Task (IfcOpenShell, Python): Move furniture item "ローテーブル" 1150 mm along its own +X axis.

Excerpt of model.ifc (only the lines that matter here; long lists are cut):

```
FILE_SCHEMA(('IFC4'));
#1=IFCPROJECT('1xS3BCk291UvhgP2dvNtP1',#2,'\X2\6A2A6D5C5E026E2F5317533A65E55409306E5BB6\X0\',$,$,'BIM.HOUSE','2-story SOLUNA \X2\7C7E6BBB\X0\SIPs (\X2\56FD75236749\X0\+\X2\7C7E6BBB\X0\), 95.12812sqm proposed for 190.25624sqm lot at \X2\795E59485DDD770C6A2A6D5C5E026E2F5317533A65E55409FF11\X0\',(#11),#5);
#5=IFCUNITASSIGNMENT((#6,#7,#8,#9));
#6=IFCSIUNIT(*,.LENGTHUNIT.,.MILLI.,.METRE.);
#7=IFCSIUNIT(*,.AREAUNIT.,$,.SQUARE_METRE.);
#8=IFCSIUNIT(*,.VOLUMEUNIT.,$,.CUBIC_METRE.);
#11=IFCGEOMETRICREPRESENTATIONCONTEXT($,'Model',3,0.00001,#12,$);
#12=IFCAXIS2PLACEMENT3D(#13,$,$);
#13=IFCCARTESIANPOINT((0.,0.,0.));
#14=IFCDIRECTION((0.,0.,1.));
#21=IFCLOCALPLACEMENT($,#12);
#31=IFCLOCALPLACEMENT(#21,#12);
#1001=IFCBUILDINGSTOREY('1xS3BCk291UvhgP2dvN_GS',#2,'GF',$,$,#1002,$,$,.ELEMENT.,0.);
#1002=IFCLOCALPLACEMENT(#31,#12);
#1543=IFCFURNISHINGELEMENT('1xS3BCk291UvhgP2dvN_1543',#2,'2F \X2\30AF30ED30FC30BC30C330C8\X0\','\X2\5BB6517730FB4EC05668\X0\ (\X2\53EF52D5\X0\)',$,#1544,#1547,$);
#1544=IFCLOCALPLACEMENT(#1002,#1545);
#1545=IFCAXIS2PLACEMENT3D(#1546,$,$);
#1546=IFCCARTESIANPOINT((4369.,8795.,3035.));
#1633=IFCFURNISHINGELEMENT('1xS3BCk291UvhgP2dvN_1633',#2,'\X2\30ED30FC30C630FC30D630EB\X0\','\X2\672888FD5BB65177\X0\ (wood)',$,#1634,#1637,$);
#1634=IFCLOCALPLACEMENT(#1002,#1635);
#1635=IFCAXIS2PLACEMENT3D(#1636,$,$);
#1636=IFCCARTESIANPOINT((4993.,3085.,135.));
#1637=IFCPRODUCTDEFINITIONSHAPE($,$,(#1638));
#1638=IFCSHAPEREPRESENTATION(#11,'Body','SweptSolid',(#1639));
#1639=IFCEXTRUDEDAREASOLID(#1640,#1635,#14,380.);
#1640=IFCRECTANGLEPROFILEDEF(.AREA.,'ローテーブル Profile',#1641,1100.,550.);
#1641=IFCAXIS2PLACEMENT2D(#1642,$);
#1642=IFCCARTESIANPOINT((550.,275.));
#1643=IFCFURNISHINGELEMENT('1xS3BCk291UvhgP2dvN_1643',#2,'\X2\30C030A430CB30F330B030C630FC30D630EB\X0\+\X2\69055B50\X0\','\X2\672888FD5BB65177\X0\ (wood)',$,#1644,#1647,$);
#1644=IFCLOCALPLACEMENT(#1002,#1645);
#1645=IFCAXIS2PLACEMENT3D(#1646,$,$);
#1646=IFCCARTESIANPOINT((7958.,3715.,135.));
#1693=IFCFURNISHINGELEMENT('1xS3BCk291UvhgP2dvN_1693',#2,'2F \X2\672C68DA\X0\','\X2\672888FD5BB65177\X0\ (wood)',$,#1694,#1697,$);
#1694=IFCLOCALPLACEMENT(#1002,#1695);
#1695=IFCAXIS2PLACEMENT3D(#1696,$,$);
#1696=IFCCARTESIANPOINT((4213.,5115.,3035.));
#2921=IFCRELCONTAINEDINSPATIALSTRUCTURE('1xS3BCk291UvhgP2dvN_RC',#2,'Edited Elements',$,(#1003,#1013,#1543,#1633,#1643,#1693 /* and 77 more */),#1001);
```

```python
import ifcopenshell
import ifcopenshell.api.geometry
import ifcopenshell.util.placement
import ifcopenshell.util.unit

model = ifcopenshell.open("model.ifc")
unit_scale = ifcopenshell.util.unit.calculate_unit_scale(model)

item = model.by_id(1633)
matrix = ifcopenshell.util.placement.get_local_placement(item.ObjectPlacement)
matrix[:3, 3] += matrix[:3, 0] * 1.15 / unit_scale
ifcopenshell.api.geometry.edit_object_placement(model, product=item, matrix=matrix, is_si=False)

print(ifcopenshell.util.placement.get_local_placement(item.ObjectPlacement).round(3) + 0.0)

model.write("model_rev.ifc")
```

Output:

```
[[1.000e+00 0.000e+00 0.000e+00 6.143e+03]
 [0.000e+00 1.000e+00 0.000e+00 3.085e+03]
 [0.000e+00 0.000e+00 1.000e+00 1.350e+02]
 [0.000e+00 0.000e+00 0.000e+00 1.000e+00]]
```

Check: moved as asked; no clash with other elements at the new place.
